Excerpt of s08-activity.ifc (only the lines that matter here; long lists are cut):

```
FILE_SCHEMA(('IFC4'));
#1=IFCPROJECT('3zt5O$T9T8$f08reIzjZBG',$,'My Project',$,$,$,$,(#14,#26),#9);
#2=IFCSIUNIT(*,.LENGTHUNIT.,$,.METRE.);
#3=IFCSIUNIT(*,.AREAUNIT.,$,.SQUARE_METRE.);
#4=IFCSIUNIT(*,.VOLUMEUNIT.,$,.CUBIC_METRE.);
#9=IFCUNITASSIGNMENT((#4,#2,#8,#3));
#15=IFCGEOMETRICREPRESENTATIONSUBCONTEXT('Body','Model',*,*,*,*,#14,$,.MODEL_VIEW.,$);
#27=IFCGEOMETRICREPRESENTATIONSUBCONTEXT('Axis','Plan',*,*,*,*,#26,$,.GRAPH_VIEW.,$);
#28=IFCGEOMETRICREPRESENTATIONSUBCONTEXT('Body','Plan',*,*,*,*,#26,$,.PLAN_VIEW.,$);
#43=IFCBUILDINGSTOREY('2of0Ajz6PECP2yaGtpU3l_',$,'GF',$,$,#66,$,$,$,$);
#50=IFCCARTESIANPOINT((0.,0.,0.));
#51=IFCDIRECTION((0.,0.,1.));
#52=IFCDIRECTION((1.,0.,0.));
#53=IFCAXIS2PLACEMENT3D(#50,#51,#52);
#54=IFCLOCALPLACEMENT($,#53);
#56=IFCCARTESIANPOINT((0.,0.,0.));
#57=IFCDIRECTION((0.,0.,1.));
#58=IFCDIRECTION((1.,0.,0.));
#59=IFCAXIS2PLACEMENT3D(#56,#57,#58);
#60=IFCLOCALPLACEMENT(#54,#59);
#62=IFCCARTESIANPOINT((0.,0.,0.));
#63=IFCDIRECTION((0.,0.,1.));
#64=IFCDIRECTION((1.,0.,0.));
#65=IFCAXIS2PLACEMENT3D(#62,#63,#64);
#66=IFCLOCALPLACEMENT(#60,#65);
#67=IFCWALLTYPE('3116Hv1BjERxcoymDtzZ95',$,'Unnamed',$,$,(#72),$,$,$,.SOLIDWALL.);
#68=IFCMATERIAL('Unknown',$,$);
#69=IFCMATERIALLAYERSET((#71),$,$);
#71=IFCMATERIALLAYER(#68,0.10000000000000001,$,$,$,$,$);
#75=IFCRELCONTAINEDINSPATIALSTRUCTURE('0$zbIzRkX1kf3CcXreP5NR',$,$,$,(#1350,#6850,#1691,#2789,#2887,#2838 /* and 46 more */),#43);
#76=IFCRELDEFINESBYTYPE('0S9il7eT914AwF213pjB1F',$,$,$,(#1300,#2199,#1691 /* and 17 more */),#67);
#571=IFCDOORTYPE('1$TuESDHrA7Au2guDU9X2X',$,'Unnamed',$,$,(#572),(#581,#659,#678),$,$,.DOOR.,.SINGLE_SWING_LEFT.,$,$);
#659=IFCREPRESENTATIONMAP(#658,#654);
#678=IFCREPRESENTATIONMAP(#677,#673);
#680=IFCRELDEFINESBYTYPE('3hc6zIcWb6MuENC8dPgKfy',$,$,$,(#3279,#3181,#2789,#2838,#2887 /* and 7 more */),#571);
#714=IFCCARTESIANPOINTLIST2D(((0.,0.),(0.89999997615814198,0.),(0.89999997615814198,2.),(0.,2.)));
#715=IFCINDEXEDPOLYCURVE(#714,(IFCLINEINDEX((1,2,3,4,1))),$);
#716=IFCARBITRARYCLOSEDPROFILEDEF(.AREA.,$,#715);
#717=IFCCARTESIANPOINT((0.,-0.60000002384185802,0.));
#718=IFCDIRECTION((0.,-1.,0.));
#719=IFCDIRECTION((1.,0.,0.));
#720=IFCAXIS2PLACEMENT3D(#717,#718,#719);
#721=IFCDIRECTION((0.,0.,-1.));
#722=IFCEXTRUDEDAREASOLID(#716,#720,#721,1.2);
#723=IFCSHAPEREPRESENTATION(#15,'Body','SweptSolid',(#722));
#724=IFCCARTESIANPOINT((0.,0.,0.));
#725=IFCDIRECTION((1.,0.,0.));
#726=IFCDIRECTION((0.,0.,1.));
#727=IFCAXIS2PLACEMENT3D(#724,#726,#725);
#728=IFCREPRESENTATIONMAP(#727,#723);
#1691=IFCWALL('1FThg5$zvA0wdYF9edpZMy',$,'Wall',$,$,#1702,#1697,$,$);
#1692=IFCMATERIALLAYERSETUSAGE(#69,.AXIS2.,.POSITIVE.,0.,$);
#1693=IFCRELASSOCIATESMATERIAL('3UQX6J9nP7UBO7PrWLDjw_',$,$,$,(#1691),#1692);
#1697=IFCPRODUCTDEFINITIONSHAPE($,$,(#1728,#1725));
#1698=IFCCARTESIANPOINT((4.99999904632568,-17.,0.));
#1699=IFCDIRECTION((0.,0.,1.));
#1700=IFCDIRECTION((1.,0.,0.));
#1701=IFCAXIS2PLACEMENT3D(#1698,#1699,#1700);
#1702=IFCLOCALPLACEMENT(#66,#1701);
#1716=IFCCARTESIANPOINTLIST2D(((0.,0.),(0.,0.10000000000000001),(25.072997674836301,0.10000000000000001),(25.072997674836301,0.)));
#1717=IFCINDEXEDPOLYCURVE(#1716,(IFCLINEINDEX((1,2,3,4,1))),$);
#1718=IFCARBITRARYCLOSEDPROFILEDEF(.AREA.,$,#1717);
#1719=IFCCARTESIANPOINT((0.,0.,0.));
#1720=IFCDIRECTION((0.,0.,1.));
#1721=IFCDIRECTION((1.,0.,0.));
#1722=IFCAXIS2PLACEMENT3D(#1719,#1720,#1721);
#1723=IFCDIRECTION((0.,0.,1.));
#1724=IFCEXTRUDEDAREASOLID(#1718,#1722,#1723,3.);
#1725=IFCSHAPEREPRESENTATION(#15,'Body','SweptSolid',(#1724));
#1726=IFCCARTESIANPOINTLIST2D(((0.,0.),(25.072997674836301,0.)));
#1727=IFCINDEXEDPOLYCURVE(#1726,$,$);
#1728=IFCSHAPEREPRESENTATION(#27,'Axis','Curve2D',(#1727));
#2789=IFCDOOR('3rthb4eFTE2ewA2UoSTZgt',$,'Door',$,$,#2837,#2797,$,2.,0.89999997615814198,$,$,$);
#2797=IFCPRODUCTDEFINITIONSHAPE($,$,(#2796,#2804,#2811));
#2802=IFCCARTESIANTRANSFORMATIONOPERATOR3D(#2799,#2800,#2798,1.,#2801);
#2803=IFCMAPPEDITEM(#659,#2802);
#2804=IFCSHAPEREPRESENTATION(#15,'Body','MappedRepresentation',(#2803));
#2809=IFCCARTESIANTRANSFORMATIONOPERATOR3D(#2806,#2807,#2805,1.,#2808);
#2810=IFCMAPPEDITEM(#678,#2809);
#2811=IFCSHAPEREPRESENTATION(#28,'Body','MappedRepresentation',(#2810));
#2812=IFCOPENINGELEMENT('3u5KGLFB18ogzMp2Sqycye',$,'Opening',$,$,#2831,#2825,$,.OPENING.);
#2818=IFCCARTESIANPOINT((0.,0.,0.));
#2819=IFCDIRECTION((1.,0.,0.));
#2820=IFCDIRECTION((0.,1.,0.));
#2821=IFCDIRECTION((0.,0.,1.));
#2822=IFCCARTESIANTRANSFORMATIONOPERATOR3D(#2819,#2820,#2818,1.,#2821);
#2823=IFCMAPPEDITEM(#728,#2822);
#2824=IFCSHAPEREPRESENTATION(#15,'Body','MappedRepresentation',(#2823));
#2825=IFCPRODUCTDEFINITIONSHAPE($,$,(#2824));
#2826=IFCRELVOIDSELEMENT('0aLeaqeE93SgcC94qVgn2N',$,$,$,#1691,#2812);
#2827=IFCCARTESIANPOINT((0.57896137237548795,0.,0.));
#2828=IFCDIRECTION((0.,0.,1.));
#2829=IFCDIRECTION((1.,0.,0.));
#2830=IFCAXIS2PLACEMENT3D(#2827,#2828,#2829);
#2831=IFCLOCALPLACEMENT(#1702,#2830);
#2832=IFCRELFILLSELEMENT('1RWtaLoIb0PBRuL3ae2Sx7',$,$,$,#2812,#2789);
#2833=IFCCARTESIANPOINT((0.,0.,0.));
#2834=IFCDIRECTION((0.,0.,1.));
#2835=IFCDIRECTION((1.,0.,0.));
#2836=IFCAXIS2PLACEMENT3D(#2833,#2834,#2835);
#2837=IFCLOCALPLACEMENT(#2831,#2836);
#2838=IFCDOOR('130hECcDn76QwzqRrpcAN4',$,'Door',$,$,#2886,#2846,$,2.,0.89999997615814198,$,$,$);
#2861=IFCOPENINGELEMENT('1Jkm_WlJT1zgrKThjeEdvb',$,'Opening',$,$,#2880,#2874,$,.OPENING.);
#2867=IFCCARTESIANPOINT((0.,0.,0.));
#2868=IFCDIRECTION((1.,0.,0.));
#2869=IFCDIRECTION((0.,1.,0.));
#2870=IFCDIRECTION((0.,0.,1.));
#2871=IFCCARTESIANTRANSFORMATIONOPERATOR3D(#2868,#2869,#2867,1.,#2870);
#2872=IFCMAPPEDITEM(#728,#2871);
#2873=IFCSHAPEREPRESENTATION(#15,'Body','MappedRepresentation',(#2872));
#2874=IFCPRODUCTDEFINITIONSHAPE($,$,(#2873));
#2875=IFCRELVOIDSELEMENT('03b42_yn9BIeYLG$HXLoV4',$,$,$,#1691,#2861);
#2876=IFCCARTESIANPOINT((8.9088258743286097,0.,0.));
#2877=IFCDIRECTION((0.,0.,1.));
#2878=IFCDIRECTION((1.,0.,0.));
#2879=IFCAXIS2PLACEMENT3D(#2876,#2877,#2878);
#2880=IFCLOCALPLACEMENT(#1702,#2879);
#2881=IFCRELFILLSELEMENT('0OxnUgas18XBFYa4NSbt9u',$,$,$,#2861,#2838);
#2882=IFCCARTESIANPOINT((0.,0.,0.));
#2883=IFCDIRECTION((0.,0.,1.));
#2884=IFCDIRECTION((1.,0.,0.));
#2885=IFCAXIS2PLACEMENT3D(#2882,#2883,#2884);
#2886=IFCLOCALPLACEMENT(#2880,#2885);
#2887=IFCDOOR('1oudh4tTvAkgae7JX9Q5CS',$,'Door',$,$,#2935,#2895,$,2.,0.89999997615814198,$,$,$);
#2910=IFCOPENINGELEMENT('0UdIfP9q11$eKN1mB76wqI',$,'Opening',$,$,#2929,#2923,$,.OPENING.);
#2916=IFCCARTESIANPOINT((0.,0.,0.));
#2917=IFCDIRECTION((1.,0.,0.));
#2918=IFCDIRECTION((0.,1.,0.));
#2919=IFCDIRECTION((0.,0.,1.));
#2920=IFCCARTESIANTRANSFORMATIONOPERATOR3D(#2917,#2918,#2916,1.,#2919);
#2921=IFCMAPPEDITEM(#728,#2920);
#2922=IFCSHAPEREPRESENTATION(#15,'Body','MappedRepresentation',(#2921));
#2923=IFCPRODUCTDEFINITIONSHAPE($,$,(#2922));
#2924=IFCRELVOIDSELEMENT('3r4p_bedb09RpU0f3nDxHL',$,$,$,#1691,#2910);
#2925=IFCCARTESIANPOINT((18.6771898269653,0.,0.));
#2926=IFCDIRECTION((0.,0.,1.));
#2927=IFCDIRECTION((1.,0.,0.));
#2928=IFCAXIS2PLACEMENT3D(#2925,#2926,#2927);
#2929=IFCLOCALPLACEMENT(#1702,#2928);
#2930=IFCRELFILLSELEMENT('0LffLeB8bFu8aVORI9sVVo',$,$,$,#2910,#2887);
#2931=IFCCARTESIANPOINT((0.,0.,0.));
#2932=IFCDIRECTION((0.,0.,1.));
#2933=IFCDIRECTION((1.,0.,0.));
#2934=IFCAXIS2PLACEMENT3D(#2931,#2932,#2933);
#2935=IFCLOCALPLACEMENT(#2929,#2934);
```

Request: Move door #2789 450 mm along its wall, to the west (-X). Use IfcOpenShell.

```python
import ifcopenshell
import ifcopenshell.api.geometry
import ifcopenshell.util.placement
import ifcopenshell.util.unit

model = ifcopenshell.open("s08-activity.ifc")
unit_scale = ifcopenshell.util.unit.calculate_unit_scale(model)

door = model.by_guid("3rthb4eFTE2ewA2UoSTZgt")
opening = door.FillsVoids[0].RelatingOpeningElement
wall = opening.VoidsElements[0].RelatingBuildingElement

wall_matrix = ifcopenshell.util.placement.get_local_placement(wall.ObjectPlacement)
shift = wall_matrix[:3, 0] * -0.45 / unit_scale
before = ifcopenshell.util.placement.get_local_placement(door.ObjectPlacement)[:3, 3].copy()

# The door is placed relative to its opening, so it follows when the opening moves.
matrix = ifcopenshell.util.placement.get_local_placement(opening.ObjectPlacement)
matrix[:3, 3] += shift
ifcopenshell.api.geometry.edit_object_placement(
    model, product=opening, matrix=matrix, is_si=False, should_transform_children=True
)

after = ifcopenshell.util.placement.get_local_placement(door.ObjectPlacement)[:3, 3]
print("door moved by", (after - before).round(3) + 0.0)

model.write("s08-activity_v2.ifc")
```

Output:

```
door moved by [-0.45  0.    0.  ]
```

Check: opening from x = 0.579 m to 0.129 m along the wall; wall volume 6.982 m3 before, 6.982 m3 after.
